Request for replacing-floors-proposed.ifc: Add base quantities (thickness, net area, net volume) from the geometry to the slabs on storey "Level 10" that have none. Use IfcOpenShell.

First a look at what the model holds.

```python
import ifcopenshell
import ifcopenshell.util.element
import ifcopenshell.util.unit

model = ifcopenshell.open("replacing-floors-proposed.ifc")
print(model.schema)
for unit_type in ("LENGTHUNIT", "AREAUNIT", "VOLUMEUNIT"):
    print(unit_type, ifcopenshell.util.unit.calculate_unit_scale(model, unit_type))
storey = next(s for s in model.by_type("IfcBuildingStorey") if s.Name == "Level 10")
slabs = [e for e in ifcopenshell.util.element.get_decomposition(storey) if e.is_a("IfcSlab")]
for e in sorted(slabs, key=lambda e: e.id()):
    print(e.id(), e.is_a(), e.Name, list(ifcopenshell.util.element.get_psets(e, qtos_only=True)), sep=" | ")
```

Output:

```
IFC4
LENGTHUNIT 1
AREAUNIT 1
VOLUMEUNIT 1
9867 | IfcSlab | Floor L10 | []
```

```python
import ifcopenshell
import ifcopenshell.api.pset
import ifcopenshell.geom
import ifcopenshell.util.element
import ifcopenshell.util.shape
import ifcopenshell.util.unit

model = ifcopenshell.open("replacing-floors-proposed.ifc")
unit_scale = ifcopenshell.util.unit.calculate_unit_scale(model)
area_scale = ifcopenshell.util.unit.calculate_unit_scale(model, "AREAUNIT")
volume_scale = ifcopenshell.util.unit.calculate_unit_scale(model, "VOLUMEUNIT")
settings = ifcopenshell.geom.settings()

storey = next(s for s in model.by_type("IfcBuildingStorey") if s.Name == "Level 10")
slabs = [e for e in ifcopenshell.util.element.get_decomposition(storey) if e.is_a("IfcSlab")]

for e in sorted(slabs, key=lambda e: e.id()):
    if ifcopenshell.util.element.get_psets(e, qtos_only=True, should_inherit=False):
        continue
    # Geometry comes back in metres, in the element's own axes.
    shape = ifcopenshell.geom.create_shape(settings, e)
    values = {
        "Width": ifcopenshell.util.shape.get_z(shape.geometry) / unit_scale,
        "NetArea": ifcopenshell.util.shape.get_footprint_area(shape.geometry) / area_scale,
        "NetVolume": ifcopenshell.util.shape.get_volume(shape.geometry) / volume_scale,
    }
    qto = ifcopenshell.api.pset.add_qto(model, product=e, name="Qto_SlabBaseQuantities")
    ifcopenshell.api.pset.edit_qto(model, qto=qto, properties=values)
    print(e.id(), {k: round(v, 3) for k, v in values.items()})

model.write("replacing-floors-proposed_updated.ifc")
```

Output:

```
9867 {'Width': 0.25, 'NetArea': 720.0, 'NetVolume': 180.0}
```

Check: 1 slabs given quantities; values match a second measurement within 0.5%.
